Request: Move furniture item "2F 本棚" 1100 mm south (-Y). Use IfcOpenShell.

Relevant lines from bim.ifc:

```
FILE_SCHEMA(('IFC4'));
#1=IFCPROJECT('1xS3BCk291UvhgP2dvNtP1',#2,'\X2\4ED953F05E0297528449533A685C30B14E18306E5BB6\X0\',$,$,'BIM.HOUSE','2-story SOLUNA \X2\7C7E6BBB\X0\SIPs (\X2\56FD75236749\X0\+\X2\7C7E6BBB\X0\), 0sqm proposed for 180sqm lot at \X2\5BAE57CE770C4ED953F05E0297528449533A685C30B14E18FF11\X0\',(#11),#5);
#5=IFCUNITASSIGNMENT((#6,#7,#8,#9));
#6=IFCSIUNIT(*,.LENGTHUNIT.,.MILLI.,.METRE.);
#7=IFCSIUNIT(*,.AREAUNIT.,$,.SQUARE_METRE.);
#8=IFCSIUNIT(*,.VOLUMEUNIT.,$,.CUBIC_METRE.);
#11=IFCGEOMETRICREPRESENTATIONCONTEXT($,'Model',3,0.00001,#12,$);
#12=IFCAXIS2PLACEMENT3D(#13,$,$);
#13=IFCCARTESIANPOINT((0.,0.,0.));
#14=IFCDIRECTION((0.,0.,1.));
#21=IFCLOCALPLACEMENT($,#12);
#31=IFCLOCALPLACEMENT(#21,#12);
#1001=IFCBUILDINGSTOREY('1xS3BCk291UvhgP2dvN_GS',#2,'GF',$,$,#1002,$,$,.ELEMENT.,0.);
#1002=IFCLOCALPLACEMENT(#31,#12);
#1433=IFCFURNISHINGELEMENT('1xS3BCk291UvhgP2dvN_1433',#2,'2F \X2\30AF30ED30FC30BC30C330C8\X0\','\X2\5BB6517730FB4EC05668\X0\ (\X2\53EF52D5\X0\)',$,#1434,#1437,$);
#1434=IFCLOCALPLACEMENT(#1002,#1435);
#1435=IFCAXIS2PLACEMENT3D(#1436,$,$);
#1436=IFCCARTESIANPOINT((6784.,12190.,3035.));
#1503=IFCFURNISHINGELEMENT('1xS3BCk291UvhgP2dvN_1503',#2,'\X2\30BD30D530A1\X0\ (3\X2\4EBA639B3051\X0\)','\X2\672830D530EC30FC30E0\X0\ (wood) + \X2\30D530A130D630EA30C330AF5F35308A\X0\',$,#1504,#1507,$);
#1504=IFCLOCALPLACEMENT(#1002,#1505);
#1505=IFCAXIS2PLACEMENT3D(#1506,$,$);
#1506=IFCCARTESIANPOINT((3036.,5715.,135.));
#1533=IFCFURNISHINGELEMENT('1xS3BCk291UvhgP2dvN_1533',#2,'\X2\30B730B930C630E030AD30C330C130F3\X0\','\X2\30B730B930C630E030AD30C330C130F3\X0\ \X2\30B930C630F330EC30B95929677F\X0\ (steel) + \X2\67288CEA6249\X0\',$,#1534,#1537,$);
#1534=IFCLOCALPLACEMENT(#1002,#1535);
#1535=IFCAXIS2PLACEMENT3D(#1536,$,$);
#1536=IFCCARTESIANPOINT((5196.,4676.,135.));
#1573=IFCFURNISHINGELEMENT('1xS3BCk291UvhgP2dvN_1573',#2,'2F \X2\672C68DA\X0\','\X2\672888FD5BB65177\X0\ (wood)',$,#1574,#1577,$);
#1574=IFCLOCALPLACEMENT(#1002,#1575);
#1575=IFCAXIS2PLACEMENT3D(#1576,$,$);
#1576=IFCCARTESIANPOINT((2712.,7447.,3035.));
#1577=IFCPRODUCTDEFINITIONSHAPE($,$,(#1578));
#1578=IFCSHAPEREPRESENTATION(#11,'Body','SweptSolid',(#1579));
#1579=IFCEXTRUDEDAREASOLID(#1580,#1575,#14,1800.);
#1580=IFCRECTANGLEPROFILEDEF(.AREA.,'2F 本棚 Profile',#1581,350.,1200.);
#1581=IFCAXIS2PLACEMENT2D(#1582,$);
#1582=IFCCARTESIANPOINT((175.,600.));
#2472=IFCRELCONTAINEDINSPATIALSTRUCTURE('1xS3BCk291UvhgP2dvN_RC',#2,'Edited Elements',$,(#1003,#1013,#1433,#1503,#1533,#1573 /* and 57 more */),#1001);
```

```python
import ifcopenshell
import ifcopenshell.api.geometry
import ifcopenshell.util.placement

model = ifcopenshell.open("bim.ifc")

item = model.by_guid("1xS3BCk291UvhgP2dvN_1573")
matrix = ifcopenshell.util.placement.get_local_placement(item.ObjectPlacement)
matrix[1, 3] -= 1100.0
ifcopenshell.api.geometry.edit_object_placement(model, product=item, matrix=matrix, is_si=False)

print(ifcopenshell.util.placement.get_local_placement(item.ObjectPlacement).round(3) + 0.0)

model.write("bim_edited.ifc")
```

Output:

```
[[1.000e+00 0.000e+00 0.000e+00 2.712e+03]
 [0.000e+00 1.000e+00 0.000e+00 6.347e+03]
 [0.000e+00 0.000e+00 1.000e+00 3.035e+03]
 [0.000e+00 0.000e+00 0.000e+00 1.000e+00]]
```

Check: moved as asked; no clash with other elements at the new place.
